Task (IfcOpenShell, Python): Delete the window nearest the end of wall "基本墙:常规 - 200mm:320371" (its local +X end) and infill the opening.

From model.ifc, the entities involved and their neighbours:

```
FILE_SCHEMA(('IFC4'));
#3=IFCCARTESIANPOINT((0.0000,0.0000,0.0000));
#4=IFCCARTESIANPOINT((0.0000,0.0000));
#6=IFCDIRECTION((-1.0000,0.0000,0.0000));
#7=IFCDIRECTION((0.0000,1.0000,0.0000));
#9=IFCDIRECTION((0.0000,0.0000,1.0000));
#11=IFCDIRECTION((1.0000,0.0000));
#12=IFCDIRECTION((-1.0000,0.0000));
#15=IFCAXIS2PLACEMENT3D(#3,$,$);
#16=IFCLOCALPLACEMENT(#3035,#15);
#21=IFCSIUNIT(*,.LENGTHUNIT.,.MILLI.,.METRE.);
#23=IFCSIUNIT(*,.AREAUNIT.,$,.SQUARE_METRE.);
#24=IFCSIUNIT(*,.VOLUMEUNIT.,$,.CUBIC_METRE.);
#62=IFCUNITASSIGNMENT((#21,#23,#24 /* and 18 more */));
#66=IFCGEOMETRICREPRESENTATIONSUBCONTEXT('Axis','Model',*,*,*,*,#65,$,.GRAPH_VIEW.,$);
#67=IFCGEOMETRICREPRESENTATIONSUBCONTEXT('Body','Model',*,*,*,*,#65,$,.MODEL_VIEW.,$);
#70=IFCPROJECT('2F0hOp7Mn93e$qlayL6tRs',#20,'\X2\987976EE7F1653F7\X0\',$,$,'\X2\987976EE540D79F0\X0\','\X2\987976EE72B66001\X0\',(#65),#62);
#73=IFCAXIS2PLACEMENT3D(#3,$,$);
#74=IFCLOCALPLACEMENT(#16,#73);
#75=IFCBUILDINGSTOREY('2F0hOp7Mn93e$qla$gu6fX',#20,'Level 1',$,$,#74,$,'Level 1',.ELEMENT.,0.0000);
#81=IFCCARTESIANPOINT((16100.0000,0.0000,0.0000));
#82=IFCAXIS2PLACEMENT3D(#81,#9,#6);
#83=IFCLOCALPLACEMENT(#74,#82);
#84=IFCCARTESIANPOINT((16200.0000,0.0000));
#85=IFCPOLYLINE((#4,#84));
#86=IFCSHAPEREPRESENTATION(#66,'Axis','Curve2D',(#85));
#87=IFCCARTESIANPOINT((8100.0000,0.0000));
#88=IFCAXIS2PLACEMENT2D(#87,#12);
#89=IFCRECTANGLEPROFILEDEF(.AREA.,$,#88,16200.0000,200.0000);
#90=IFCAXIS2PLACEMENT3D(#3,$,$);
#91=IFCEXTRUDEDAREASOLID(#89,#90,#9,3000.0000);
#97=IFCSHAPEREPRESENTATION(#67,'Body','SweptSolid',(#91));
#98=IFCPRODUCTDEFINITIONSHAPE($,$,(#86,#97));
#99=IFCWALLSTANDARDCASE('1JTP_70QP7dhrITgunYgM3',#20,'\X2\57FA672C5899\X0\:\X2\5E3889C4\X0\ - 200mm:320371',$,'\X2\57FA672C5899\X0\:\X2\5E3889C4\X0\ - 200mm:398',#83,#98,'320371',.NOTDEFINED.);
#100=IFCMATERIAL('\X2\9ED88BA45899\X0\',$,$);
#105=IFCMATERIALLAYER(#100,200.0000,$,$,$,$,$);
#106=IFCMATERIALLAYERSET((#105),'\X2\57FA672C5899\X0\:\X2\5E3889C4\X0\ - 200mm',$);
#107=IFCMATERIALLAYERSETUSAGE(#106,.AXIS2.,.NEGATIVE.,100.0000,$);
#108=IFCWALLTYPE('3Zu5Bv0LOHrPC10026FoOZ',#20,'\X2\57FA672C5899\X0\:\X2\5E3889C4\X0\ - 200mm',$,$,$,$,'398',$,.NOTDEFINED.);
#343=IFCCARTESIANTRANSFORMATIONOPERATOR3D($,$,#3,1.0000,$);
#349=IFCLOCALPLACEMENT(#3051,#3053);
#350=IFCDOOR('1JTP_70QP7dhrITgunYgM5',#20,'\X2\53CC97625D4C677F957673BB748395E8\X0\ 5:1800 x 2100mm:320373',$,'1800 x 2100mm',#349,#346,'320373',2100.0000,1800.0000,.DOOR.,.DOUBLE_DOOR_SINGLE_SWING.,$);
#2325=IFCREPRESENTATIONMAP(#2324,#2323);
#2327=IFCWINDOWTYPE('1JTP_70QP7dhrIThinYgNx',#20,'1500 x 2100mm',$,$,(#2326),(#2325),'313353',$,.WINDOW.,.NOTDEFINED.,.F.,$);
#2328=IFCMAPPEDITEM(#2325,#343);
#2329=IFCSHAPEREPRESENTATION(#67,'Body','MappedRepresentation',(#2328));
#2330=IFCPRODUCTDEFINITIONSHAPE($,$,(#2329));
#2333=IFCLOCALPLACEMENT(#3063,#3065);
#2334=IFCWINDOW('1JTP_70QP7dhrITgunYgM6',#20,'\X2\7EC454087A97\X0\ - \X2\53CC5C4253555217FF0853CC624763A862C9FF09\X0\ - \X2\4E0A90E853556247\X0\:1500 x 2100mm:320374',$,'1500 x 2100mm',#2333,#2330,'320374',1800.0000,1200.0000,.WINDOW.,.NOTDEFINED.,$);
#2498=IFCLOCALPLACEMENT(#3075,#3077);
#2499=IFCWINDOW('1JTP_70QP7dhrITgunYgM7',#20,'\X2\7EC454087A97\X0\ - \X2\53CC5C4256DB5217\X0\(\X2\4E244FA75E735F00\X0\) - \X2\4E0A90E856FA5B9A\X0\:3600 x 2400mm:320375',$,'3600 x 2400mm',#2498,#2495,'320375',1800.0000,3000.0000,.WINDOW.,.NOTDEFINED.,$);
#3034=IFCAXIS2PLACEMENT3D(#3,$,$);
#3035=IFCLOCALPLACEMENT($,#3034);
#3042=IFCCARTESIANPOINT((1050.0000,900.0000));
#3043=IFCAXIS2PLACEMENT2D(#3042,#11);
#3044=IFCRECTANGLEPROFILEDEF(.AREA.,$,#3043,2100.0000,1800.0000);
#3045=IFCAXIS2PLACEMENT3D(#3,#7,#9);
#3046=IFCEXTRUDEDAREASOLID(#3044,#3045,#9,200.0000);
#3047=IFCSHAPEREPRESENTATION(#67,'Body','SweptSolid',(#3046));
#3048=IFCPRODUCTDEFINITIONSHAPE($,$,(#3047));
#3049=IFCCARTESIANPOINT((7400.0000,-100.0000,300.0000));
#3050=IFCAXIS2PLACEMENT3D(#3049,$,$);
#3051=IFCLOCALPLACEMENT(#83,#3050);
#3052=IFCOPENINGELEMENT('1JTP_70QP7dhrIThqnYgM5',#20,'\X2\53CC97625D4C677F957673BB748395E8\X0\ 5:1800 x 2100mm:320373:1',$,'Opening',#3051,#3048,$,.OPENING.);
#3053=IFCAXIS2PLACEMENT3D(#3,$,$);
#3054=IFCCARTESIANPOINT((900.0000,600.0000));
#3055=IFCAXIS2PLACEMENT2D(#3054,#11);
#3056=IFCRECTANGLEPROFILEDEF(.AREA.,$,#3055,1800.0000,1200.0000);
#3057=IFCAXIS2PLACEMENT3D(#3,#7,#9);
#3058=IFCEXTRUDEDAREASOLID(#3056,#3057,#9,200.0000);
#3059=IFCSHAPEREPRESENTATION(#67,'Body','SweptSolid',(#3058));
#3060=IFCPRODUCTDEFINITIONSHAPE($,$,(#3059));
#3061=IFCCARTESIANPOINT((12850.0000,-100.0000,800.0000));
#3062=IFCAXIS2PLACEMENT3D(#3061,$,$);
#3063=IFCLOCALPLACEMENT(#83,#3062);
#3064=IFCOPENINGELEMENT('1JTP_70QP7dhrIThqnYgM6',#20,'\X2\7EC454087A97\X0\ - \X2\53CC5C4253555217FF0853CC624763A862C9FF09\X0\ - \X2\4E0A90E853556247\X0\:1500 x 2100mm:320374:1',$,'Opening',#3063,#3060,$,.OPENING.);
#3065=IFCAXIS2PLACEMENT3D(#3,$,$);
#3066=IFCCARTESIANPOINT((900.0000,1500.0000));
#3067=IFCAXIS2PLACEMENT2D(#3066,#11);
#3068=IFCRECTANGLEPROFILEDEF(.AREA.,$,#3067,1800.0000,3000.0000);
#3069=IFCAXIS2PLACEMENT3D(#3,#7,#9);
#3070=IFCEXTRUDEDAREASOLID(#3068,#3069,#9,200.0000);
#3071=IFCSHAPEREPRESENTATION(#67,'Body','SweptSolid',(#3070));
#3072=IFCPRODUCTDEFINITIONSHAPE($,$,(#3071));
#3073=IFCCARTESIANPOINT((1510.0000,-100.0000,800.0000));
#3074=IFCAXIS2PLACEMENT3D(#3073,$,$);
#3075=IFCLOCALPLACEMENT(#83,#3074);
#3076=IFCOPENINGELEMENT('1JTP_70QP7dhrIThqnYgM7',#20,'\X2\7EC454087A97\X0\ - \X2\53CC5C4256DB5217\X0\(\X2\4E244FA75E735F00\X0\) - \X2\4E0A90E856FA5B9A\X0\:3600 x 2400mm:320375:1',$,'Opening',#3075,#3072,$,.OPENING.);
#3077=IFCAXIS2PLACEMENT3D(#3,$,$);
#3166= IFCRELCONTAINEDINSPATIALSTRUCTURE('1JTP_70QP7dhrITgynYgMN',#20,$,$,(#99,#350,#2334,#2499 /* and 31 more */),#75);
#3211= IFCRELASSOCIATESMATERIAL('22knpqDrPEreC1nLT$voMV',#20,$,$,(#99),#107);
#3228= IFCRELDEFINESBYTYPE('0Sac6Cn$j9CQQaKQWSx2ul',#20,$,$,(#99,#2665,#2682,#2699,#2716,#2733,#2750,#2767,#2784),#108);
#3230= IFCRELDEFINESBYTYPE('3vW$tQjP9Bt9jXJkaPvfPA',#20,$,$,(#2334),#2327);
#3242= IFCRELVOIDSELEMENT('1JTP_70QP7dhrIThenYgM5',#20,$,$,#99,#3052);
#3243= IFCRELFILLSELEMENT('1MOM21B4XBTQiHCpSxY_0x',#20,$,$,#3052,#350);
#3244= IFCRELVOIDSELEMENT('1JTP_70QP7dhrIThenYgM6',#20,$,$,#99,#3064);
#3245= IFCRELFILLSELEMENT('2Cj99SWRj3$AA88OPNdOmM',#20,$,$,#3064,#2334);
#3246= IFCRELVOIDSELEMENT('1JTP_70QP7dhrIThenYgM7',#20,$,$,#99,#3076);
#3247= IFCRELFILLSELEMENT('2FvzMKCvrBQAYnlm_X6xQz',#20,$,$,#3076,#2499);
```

```python
import ifcopenshell
import ifcopenshell.api.feature
import ifcopenshell.api.root
import ifcopenshell.geom
import ifcopenshell.util.shape

model = ifcopenshell.open("model.ifc")
settings = ifcopenshell.geom.settings()


def volume(element):
    """Net volume in cubic metres, openings subtracted."""
    shape = ifcopenshell.geom.create_shape(settings, element)
    return ifcopenshell.util.shape.get_volume(shape.geometry)


window = model.by_guid("1JTP_70QP7dhrITgunYgM6")
opening = window.FillsVoids[0].RelatingOpeningElement
wall = opening.VoidsElements[0].RelatingBuildingElement
before = volume(wall)

ifcopenshell.api.root.remove_product(model, product=window)
ifcopenshell.api.feature.remove_feature(model, feature=opening)

after = volume(wall)

print(f"wall volume {before:.3f} -> {after:.3f} m3")

model.write("model_v2.ifc")
```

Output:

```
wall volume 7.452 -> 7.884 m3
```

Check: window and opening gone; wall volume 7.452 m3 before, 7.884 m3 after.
